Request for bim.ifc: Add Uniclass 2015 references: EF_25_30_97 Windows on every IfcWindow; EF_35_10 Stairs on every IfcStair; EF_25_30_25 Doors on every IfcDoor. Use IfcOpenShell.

First a look at what the model holds.

```python
import ifcopenshell

model = ifcopenshell.open("bim.ifc")
print(model.schema)
print("classifications:", [c.Name for c in model.by_type("IfcClassification")])
for ifc_class in ("IfcDoor", "IfcRoof", "IfcStair", "IfcWall", "IfcWindow"):
    print(ifc_class, len(model.by_type(ifc_class)))
```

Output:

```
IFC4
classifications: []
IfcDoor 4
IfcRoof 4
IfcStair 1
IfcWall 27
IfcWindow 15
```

```python
import ifcopenshell
import ifcopenshell.api.classification

model = ifcopenshell.open("bim.ifc")

system = ifcopenshell.api.classification.add_classification(model, classification="Uniclass 2015")

codes = {
    "IfcWindow": ("EF_25_30_97", "Windows"),
    "IfcStair": ("EF_35_10", "Stairs"),
    "IfcDoor": ("EF_25_30_25", "Doors"),
}
for ifc_class, (code, name) in codes.items():
    products = model.by_type(ifc_class)
    ifcopenshell.api.classification.add_reference(
        model, products=products, classification=system, identification=code, name=name
    )
    print(code, len(products))

model.write("bim_updated.ifc")
```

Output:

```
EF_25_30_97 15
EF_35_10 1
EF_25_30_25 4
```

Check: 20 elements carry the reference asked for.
